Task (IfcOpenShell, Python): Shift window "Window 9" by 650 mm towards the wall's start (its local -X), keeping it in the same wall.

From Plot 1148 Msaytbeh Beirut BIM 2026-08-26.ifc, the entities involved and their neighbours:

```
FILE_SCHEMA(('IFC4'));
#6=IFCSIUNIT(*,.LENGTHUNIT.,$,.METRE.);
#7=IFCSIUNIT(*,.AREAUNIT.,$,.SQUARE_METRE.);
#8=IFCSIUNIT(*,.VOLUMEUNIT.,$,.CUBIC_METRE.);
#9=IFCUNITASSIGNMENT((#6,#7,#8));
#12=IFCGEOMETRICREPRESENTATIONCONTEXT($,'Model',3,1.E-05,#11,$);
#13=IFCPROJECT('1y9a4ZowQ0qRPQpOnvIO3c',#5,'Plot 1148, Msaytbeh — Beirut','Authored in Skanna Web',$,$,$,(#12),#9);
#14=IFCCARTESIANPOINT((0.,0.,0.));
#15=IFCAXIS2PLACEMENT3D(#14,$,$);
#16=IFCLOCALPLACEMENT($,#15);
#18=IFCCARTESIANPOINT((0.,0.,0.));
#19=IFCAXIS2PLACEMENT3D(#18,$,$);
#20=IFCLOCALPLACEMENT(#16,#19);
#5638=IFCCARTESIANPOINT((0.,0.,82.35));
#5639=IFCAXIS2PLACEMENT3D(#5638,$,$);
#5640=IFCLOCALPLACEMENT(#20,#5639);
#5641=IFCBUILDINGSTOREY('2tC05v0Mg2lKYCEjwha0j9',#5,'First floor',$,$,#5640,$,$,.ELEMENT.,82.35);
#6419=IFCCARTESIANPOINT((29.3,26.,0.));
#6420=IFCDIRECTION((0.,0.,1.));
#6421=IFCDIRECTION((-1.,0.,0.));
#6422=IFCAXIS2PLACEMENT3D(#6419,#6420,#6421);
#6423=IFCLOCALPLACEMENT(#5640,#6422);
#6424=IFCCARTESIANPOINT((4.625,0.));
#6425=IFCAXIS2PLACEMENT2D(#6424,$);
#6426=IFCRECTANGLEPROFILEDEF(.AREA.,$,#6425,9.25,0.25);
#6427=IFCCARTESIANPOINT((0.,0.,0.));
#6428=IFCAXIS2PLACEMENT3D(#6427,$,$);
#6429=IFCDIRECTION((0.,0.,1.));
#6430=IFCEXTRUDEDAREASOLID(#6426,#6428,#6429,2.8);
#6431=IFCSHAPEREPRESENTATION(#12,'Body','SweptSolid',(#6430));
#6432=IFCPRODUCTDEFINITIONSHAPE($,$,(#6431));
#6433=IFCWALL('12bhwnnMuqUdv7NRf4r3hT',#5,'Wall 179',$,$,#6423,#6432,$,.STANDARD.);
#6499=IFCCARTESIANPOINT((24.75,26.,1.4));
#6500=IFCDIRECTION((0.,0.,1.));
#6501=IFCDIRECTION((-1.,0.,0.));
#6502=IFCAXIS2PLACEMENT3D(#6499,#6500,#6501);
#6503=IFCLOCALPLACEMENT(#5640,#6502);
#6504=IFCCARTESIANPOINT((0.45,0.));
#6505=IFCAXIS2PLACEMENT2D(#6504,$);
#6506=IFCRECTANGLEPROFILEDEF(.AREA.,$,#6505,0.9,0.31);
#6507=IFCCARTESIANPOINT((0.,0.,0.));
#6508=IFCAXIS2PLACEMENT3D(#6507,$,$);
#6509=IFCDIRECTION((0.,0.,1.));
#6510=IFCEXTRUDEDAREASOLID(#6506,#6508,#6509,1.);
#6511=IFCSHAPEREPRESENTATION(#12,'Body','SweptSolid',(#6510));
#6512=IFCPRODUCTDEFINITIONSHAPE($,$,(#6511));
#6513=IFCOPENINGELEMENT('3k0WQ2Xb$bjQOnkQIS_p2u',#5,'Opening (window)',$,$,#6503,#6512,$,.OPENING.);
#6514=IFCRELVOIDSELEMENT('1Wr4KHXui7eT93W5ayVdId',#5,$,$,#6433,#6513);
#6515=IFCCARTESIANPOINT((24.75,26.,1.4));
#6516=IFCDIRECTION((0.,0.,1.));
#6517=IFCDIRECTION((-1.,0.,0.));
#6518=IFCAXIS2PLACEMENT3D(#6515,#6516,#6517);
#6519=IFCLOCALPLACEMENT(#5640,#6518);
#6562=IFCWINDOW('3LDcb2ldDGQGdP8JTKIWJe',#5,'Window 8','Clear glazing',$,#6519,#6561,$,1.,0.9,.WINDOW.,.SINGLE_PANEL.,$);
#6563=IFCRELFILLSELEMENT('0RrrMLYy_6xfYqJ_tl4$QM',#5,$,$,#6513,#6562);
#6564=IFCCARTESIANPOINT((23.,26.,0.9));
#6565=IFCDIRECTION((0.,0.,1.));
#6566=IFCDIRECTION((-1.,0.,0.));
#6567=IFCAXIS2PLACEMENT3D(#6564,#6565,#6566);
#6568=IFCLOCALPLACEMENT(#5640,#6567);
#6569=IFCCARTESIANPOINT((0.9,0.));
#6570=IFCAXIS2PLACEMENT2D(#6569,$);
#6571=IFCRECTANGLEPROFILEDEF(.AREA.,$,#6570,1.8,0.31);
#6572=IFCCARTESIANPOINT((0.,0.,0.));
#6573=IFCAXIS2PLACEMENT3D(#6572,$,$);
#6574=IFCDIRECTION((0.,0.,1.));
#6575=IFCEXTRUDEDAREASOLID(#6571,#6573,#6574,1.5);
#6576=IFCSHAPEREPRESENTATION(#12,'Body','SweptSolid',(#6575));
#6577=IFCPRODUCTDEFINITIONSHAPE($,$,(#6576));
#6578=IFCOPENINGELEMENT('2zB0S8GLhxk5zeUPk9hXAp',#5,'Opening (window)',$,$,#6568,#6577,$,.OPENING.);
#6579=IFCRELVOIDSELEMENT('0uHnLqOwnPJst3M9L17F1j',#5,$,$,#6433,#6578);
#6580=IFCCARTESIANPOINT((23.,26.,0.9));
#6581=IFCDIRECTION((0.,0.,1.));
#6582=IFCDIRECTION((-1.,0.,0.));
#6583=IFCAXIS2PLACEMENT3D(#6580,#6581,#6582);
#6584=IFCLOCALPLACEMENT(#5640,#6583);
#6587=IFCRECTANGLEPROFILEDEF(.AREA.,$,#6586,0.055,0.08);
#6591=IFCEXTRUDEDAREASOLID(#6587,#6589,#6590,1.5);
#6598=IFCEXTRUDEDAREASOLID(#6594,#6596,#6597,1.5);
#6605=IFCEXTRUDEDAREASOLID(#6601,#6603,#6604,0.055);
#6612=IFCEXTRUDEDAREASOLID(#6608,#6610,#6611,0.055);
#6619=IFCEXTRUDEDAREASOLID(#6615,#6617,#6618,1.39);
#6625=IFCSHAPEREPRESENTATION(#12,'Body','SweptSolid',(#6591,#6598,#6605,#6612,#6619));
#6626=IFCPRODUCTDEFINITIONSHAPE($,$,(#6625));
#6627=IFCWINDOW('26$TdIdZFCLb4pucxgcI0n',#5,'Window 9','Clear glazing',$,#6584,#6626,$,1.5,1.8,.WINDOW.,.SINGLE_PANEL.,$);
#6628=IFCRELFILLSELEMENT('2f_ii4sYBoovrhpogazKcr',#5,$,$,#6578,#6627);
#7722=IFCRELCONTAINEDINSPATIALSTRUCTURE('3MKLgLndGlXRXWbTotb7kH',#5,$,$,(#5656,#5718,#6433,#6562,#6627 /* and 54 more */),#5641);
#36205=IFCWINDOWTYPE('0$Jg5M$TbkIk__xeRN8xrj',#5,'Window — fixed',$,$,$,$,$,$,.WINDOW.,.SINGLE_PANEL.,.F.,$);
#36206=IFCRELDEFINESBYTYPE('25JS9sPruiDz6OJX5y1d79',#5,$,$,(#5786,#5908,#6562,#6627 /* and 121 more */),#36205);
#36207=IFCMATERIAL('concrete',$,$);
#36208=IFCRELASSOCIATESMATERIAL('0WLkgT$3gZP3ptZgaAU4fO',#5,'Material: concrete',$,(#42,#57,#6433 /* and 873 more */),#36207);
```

```python
import ifcopenshell
import ifcopenshell.api.geometry
import ifcopenshell.util.placement

model = ifcopenshell.open("Plot 1148 Msaytbeh Beirut BIM 2026-08-26.ifc")

window = model.by_guid("26$TdIdZFCLb4pucxgcI0n")
opening = window.FillsVoids[0].RelatingOpeningElement
wall = opening.VoidsElements[0].RelatingBuildingElement

wall_matrix = ifcopenshell.util.placement.get_local_placement(wall.ObjectPlacement)
shift = wall_matrix[:3, 0] * -0.65
before = ifcopenshell.util.placement.get_local_placement(window.ObjectPlacement)[:3, 3].copy()

# The window is not placed relative to its opening, so move both.
for product in (opening, window):
    matrix = ifcopenshell.util.placement.get_local_placement(product.ObjectPlacement)
    matrix[:3, 3] += shift
    ifcopenshell.api.geometry.edit_object_placement(model, product=product, matrix=matrix, is_si=False)

after = ifcopenshell.util.placement.get_local_placement(window.ObjectPlacement)[:3, 3]
print("window moved by", (after - before).round(3) + 0.0)

model.write("Plot 1148 Msaytbeh Beirut BIM 2026-08-26-out.ifc")
```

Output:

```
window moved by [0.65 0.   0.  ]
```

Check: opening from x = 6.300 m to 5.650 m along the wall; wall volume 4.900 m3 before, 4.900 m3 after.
